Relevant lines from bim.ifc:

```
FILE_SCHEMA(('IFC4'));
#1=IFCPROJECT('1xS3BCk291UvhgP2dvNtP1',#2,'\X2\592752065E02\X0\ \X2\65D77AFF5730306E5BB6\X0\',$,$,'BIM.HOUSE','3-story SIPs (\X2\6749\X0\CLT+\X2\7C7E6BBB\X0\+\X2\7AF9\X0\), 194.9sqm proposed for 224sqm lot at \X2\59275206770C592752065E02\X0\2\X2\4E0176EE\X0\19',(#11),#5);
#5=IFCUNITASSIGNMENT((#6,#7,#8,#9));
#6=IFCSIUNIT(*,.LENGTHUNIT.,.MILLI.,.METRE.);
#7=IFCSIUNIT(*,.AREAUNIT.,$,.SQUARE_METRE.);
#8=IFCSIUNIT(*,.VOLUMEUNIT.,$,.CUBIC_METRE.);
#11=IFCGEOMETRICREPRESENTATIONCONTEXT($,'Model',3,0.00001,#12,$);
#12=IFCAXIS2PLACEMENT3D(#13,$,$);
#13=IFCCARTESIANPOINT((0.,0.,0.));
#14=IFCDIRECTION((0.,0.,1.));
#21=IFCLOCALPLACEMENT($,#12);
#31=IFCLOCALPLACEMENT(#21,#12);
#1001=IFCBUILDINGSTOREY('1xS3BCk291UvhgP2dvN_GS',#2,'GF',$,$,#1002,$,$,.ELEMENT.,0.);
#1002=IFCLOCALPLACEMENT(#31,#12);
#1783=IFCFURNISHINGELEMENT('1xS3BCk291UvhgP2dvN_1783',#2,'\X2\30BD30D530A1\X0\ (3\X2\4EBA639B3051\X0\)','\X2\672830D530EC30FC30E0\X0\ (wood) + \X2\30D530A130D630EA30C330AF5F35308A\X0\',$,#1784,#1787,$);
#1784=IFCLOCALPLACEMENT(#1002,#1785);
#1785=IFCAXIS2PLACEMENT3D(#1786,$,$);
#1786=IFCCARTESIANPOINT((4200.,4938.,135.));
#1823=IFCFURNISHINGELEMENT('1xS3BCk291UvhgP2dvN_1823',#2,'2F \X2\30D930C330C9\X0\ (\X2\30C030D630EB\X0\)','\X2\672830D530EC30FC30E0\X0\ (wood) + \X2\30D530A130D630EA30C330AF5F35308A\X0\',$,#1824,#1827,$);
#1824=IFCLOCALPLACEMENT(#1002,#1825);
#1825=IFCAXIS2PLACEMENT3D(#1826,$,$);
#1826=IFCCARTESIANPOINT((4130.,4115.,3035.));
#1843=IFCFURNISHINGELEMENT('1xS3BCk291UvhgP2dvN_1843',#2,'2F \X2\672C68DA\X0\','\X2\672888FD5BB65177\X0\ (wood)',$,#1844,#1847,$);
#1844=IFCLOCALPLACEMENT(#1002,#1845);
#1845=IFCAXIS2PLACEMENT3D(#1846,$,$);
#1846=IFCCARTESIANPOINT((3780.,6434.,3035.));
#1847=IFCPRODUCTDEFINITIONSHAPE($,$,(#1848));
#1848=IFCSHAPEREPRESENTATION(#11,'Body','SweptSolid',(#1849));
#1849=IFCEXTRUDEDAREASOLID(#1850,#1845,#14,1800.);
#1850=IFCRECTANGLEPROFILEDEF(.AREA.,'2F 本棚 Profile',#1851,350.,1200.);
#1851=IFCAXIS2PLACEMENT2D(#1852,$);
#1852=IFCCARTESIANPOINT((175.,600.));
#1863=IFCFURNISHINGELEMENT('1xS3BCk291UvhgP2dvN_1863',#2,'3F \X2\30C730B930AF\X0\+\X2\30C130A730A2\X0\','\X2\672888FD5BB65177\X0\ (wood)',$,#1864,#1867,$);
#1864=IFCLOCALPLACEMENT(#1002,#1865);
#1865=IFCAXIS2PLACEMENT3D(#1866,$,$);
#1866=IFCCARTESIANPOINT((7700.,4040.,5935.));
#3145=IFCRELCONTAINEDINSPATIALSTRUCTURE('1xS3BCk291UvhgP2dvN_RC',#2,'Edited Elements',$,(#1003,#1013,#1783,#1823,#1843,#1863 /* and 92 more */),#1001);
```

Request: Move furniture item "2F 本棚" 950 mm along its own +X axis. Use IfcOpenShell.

```python
import ifcopenshell
import ifcopenshell.api.geometry
import ifcopenshell.util.placement
import ifcopenshell.util.unit

model = ifcopenshell.open("bim.ifc")
unit_scale = ifcopenshell.util.unit.calculate_unit_scale(model)

item = model.by_guid("1xS3BCk291UvhgP2dvN_1843")
matrix = ifcopenshell.util.placement.get_local_placement(item.ObjectPlacement)
matrix[:3, 3] += matrix[:3, 0] * 0.95 / unit_scale
ifcopenshell.api.geometry.edit_object_placement(model, product=item, matrix=matrix, is_si=False)

print(ifcopenshell.util.placement.get_local_placement(item.ObjectPlacement).round(3) + 0.0)

model.write("bim_v2.ifc")
```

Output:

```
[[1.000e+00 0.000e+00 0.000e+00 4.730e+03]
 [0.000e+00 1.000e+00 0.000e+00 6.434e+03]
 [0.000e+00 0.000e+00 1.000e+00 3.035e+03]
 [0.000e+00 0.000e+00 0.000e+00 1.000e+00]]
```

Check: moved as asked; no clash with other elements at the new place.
